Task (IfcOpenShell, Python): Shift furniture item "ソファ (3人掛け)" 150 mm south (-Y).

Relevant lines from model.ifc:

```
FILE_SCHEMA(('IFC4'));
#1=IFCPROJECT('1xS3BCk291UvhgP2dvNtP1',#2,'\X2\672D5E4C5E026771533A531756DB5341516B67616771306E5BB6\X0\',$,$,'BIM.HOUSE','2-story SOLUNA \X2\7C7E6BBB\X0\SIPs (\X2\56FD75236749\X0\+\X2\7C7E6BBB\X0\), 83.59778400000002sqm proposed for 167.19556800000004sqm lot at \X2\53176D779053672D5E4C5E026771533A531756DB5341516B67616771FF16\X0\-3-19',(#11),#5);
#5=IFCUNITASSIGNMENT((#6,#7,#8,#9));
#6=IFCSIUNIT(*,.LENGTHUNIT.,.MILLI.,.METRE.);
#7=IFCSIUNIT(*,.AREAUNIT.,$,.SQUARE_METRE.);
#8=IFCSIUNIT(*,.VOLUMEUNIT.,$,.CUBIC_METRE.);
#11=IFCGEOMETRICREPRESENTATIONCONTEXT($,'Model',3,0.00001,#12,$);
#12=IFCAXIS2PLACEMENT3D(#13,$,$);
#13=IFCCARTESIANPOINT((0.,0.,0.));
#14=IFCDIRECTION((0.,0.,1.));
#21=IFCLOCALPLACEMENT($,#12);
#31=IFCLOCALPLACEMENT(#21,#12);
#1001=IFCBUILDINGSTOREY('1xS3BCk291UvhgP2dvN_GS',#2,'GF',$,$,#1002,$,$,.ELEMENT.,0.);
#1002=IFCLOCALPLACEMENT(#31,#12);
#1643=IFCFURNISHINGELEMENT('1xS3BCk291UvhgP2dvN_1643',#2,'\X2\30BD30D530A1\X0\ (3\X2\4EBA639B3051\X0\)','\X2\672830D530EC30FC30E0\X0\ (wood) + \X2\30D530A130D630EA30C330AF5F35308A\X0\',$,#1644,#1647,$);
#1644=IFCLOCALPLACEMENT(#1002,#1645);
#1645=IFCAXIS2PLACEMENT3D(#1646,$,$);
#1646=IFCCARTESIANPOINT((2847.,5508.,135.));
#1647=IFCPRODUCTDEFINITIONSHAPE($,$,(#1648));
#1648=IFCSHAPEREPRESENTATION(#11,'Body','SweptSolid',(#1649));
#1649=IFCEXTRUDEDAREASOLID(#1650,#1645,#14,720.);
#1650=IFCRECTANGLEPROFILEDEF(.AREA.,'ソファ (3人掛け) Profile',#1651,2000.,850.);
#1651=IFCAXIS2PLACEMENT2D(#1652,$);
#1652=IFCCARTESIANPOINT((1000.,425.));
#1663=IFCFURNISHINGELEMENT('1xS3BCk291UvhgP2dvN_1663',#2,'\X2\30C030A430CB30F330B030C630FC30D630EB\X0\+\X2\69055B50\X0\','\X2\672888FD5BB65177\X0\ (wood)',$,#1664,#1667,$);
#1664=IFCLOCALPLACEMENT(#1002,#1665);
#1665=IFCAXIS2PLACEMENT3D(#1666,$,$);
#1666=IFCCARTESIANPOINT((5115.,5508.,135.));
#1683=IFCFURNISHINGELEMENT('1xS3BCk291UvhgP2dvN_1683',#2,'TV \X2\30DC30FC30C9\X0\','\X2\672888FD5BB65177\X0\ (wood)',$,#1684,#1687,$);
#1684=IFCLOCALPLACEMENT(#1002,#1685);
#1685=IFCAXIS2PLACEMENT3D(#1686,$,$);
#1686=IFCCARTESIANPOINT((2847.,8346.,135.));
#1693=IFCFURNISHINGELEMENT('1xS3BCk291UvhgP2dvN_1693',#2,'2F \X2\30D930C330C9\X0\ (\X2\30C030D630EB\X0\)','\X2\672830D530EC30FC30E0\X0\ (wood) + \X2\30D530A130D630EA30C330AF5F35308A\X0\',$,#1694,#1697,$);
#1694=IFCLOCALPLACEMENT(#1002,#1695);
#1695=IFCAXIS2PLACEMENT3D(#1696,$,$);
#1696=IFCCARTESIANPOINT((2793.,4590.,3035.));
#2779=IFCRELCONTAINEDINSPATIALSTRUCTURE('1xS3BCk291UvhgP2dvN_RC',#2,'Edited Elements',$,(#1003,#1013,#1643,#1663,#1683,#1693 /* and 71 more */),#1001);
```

```python
import ifcopenshell
import ifcopenshell.api.geometry
import ifcopenshell.util.placement
import ifcopenshell.util.unit

model = ifcopenshell.open("model.ifc")
unit_scale = ifcopenshell.util.unit.calculate_unit_scale(model)

item = model.by_guid("1xS3BCk291UvhgP2dvN_1643")
matrix = ifcopenshell.util.placement.get_local_placement(item.ObjectPlacement)
matrix[1, 3] -= 0.15 / unit_scale
ifcopenshell.api.geometry.edit_object_placement(model, product=item, matrix=matrix, is_si=False)

print(ifcopenshell.util.placement.get_local_placement(item.ObjectPlacement).round(3) + 0.0)

model.write("model_edited.ifc")
```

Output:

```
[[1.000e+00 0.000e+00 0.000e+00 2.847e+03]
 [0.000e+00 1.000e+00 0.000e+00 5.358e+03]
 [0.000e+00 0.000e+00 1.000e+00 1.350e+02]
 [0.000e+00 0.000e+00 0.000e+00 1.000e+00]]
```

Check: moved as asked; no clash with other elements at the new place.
